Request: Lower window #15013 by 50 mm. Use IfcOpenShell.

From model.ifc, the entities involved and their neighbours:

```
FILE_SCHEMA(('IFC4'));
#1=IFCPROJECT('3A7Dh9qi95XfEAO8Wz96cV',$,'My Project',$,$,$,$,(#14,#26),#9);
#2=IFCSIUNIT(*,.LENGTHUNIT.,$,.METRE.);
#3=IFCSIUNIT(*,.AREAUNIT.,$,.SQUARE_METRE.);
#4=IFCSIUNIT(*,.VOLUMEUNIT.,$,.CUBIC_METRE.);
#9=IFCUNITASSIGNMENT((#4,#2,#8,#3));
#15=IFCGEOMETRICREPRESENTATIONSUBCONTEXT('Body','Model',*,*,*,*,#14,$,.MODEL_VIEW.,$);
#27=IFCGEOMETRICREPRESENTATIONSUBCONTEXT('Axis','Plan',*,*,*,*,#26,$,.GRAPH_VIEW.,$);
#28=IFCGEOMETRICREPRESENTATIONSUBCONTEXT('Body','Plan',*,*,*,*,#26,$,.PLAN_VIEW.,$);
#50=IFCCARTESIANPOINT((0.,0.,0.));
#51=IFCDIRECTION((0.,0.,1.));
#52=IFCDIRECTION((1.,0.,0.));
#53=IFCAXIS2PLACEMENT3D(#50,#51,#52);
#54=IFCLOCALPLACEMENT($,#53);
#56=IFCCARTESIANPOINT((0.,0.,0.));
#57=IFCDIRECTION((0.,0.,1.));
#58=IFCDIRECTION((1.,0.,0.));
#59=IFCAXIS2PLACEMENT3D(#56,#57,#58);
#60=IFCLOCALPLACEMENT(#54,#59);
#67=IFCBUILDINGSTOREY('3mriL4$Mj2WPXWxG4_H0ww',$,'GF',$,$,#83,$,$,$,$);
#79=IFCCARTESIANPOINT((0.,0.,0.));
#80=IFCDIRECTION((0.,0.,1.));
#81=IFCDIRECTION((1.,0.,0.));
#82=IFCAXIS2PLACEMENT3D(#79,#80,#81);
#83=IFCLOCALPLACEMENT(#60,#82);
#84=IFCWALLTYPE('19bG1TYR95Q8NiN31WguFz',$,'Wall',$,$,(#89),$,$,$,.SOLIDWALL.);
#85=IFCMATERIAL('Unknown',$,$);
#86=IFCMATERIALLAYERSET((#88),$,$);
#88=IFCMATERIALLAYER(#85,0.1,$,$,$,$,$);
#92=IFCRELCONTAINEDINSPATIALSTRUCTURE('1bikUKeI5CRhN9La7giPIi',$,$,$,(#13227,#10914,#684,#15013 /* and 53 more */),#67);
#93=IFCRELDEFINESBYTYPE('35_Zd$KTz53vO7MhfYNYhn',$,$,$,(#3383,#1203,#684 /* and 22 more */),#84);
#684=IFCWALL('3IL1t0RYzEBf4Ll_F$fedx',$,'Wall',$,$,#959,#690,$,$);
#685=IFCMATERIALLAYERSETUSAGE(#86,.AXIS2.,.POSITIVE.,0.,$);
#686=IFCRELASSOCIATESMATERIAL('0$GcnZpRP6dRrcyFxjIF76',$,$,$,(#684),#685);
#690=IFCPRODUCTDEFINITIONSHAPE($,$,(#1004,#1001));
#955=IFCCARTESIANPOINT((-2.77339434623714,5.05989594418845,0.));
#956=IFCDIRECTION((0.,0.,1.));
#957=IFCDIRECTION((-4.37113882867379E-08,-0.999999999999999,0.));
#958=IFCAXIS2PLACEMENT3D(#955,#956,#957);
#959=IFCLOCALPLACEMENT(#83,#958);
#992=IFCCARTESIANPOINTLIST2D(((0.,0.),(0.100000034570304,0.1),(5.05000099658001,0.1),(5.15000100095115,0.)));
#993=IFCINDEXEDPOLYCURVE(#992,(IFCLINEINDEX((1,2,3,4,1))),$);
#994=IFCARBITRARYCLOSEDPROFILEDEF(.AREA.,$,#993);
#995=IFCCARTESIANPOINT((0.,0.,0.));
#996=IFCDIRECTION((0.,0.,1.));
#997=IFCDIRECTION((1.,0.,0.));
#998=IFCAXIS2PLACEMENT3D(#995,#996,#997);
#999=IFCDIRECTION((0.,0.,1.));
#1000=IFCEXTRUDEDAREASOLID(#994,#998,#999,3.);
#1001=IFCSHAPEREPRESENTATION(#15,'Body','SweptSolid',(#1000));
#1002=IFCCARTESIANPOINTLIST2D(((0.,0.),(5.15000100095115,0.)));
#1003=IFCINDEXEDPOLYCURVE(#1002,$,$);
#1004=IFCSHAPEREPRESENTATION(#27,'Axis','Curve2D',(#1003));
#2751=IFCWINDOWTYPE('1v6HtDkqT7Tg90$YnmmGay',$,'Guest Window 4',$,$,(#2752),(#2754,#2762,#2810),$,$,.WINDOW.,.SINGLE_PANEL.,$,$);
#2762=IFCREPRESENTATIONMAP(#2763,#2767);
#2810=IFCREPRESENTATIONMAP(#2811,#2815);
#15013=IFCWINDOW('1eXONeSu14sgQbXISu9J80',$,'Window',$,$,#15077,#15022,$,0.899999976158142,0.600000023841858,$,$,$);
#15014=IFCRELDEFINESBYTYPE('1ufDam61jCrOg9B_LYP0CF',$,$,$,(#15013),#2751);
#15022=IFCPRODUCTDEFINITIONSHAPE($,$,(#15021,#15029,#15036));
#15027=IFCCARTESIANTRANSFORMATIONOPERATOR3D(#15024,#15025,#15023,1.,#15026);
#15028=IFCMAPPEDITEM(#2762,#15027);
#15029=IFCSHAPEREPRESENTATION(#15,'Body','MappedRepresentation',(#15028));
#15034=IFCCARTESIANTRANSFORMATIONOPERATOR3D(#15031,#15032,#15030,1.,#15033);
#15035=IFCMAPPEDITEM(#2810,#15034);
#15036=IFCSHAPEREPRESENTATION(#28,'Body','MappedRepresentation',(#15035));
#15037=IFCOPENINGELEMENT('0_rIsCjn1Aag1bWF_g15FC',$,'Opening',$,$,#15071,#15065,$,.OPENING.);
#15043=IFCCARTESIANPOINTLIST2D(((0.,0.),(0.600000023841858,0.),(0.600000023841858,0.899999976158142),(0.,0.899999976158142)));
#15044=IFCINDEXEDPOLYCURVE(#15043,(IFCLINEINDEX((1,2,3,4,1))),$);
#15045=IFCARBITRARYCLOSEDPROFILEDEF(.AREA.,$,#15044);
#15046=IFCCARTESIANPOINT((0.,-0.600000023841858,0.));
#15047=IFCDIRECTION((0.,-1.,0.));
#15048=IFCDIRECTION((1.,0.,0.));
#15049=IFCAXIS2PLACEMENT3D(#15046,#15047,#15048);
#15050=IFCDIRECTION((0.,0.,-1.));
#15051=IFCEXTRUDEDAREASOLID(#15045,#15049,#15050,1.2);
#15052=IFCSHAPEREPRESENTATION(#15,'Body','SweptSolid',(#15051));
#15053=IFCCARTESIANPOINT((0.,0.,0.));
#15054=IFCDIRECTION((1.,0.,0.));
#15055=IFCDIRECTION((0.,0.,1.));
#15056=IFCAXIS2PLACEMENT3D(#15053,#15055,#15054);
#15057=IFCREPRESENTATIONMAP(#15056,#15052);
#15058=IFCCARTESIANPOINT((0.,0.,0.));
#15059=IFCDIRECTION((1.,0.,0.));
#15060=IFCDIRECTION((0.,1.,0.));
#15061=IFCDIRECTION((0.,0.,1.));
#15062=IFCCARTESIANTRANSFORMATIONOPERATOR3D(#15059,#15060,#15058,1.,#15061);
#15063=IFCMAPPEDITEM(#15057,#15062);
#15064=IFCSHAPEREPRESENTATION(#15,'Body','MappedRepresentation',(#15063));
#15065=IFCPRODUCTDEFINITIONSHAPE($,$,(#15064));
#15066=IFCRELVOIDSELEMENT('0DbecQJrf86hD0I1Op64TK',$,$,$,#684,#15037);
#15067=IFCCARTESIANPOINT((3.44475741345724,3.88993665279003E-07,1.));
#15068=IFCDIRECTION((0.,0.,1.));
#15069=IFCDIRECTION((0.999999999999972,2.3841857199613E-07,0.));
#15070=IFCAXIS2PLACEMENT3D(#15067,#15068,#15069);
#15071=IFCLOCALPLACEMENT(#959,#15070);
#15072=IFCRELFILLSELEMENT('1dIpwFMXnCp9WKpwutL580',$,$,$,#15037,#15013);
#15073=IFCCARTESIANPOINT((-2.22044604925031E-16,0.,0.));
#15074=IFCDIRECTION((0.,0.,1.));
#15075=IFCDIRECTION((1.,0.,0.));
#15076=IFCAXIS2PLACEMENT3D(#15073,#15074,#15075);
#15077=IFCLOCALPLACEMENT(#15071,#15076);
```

```python
import numpy as np
import ifcopenshell
import ifcopenshell.api.geometry
import ifcopenshell.util.placement
import ifcopenshell.util.unit

model = ifcopenshell.open("model.ifc")
unit_scale = ifcopenshell.util.unit.calculate_unit_scale(model)

window = model.by_guid("1eXONeSu14sgQbXISu9J80")
opening = window.FillsVoids[0].RelatingOpeningElement
dz = -0.05 / unit_scale

shift = np.array([0.0, 0.0, dz])
# The window is placed relative to its opening, so it follows when the opening moves.
matrix = ifcopenshell.util.placement.get_local_placement(opening.ObjectPlacement)
matrix[:3, 3] += shift
ifcopenshell.api.geometry.edit_object_placement(
    model, product=opening, matrix=matrix, is_si=False, should_transform_children=True
)

print(f"moved by {dz * unit_scale:+.3f} m")

model.write("model_v2.ifc")
```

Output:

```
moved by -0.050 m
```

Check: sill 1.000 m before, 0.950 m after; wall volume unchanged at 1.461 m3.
